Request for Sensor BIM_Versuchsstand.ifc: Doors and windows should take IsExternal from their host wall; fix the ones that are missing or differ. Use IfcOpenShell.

First a look at what the model holds.

```python
import ifcopenshell
import ifcopenshell.util.element

model = ifcopenshell.open("Sensor BIM_Versuchsstand.ifc")
print(model.schema)
seen = {}
for e in model.by_type("IfcDoor") + model.by_type("IfcWindow"):
    if not e.FillsVoids:
        continue
    host = e.FillsVoids[0].RelatingOpeningElement.VoidsElements[0].RelatingBuildingElement
    own = ifcopenshell.util.element.get_pset(e, f"Pset_{e.is_a()[3:].removesuffix('StandardCase')}Common", "IsExternal")
    wall = ifcopenshell.util.element.get_pset(host, "Pset_WallCommon", "IsExternal")
    seen[e.is_a(), own, wall] = seen.get((e.is_a(), own, wall), 0) + 1
for (cls, own, wall), count in sorted(seen.items(), key=str):
    print(count, cls, "IsExternal:", own, "| host wall:", wall)
```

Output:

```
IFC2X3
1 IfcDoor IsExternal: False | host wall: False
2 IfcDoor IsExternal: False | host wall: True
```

```python
import ifcopenshell
import ifcopenshell.api.pset
import ifcopenshell.util.element

model = ifcopenshell.open("Sensor BIM_Versuchsstand.ifc")

count = 0
for ifc_class, pset_name in (("IfcDoor", "Pset_DoorCommon"), ("IfcWindow", "Pset_WindowCommon")):
    for e in model.by_type(ifc_class):
        if not e.FillsVoids:
            continue
        host = e.FillsVoids[0].RelatingOpeningElement.VoidsElements[0].RelatingBuildingElement
        external = ifcopenshell.util.element.get_pset(host, "Pset_WallCommon", "IsExternal")
        if external is None or ifcopenshell.util.element.get_pset(e, pset_name, "IsExternal") == external:
            continue
        pset = ifcopenshell.api.pset.add_pset(model, product=e, name=pset_name)
        ifcopenshell.api.pset.edit_pset(model, pset=pset, properties={"IsExternal": external})
        count += 1

print(count, "updated")

model.write("Sensor BIM_Versuchsstand-out.ifc")
```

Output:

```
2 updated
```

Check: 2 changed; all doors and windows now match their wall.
